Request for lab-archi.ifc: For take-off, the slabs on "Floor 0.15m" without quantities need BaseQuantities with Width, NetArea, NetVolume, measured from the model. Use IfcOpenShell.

First a look at what the model holds.

```python
import ifcopenshell
import ifcopenshell.util.element
import ifcopenshell.util.unit

model = ifcopenshell.open("lab-archi.ifc")
print(model.schema)
for unit_type in ("LENGTHUNIT", "AREAUNIT", "VOLUMEUNIT"):
    print(unit_type, ifcopenshell.util.unit.calculate_unit_scale(model, unit_type))
storey = next(s for s in model.by_type("IfcBuildingStorey") if s.Name == "Floor 0.15m")
slabs = [e for e in ifcopenshell.util.element.get_decomposition(storey) if e.is_a("IfcSlab")]
for e in sorted(slabs, key=lambda e: e.id()):
    print(e.id(), e.is_a(), e.Name, list(ifcopenshell.util.element.get_psets(e, qtos_only=True)), sep=" | ")
```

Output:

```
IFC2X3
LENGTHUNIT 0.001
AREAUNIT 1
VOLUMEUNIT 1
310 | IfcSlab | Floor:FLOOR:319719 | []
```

```python
import ifcopenshell
import ifcopenshell.api.pset
import ifcopenshell.geom
import ifcopenshell.util.element
import ifcopenshell.util.shape
import ifcopenshell.util.unit

model = ifcopenshell.open("lab-archi.ifc")
unit_scale = ifcopenshell.util.unit.calculate_unit_scale(model)
area_scale = ifcopenshell.util.unit.calculate_unit_scale(model, "AREAUNIT")
volume_scale = ifcopenshell.util.unit.calculate_unit_scale(model, "VOLUMEUNIT")
settings = ifcopenshell.geom.settings()

storey = next(s for s in model.by_type("IfcBuildingStorey") if s.Name == "Floor 0.15m")
slabs = [e for e in ifcopenshell.util.element.get_decomposition(storey) if e.is_a("IfcSlab")]

for e in sorted(slabs, key=lambda e: e.id()):
    if ifcopenshell.util.element.get_psets(e, qtos_only=True, should_inherit=False):
        continue
    # Geometry comes back in metres, in the element's own axes.
    shape = ifcopenshell.geom.create_shape(settings, e)
    values = {
        "Width": ifcopenshell.util.shape.get_z(shape.geometry) / unit_scale,
        "NetArea": ifcopenshell.util.shape.get_footprint_area(shape.geometry) / area_scale,
        "NetVolume": ifcopenshell.util.shape.get_volume(shape.geometry) / volume_scale,
    }
    qto = ifcopenshell.api.pset.add_qto(model, product=e, name="BaseQuantities")
    ifcopenshell.api.pset.edit_qto(model, qto=qto, properties=values)
    print(e.id(), {k: round(v, 3) for k, v in values.items()})

model.write("lab-archi_rev.ifc")
```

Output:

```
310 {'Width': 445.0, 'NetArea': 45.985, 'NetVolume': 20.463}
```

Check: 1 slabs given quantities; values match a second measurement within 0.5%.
